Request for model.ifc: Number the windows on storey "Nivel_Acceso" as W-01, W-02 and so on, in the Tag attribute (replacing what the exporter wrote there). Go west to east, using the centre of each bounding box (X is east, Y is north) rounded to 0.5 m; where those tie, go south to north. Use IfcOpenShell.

First a look at what the model holds.

```python
import ifcopenshell
import ifcopenshell.util.element
import ifcopenshell.util.placement

model = ifcopenshell.open("model.ifc")
print(model.schema)
storey = next(s for s in model.by_type("IfcBuildingStorey") if s.Name == "Nivel_Acceso")
windows = [e for e in ifcopenshell.util.element.get_decomposition(storey) if e.is_a("IfcWindow")]
for e in sorted(windows, key=lambda e: e.id()):
    origin = ifcopenshell.util.placement.get_local_placement(e.ObjectPlacement)[:3, 3]
    print(e.id(), e.Tag, e.Name, origin.round(2) + 0.0, sep=" | ")
```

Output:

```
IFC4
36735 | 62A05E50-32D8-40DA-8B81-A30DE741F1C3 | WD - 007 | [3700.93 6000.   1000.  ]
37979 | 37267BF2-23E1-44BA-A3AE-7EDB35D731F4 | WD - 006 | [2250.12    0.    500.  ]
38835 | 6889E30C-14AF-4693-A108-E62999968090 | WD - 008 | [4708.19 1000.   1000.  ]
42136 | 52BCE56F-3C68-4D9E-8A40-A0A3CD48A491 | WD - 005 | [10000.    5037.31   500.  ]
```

```python
import ifcopenshell
import ifcopenshell.geom
import ifcopenshell.util.element
import ifcopenshell.util.shape

model = ifcopenshell.open("model.ifc")
settings = ifcopenshell.geom.settings()
settings.set("use-world-coords", True)


def centre(element):
    shape = ifcopenshell.geom.create_shape(settings, element)
    return ifcopenshell.util.shape.get_bbox_centroid(shape.geometry)


storey = next(s for s in model.by_type("IfcBuildingStorey") if s.Name == "Nivel_Acceso")
windows = [e for e in ifcopenshell.util.element.get_decomposition(storey) if e.is_a("IfcWindow")]

# Insertion points can sit at a corner or the storey origin, so sort by the geometry (in metres).
centres = {e: centre(e) for e in windows}
windows.sort(key=lambda e: (round(centres[e][0] / 0.5), centres[e][1]))

for i, e in enumerate(windows, start=1):
    number = f"W-{i:02d}"
    e.Tag = number
    print(e.id(), number)

model.write("model_rev.ifc")
```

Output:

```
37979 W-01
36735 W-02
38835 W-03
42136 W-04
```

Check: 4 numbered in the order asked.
